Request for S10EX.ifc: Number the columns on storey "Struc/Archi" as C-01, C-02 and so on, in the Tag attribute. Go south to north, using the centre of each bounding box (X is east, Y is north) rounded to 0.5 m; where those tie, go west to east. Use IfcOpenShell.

First a look at what the model holds.

```python
import ifcopenshell
import ifcopenshell.util.element
import ifcopenshell.util.placement

model = ifcopenshell.open("S10EX.ifc")
print(model.schema)
storey = next(s for s in model.by_type("IfcBuildingStorey") if s.Name == "Struc/Archi")
columns = [e for e in ifcopenshell.util.element.get_decomposition(storey) if e.is_a("IfcColumn")]
for e in sorted(columns, key=lambda e: e.id()):
    origin = ifcopenshell.util.placement.get_local_placement(e.ObjectPlacement)[:3, 3]
    print(e.id(), e.Tag, e.Name, origin.round(2) + 0.0, sep=" | ")
```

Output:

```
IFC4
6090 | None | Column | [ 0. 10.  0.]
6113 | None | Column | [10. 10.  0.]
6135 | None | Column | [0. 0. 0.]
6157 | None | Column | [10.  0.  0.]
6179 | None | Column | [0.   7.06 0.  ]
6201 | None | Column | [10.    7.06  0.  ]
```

```python
import ifcopenshell
import ifcopenshell.geom
import ifcopenshell.util.element
import ifcopenshell.util.shape

model = ifcopenshell.open("S10EX.ifc")
settings = ifcopenshell.geom.settings()
settings.set("use-world-coords", True)


def centre(element):
    shape = ifcopenshell.geom.create_shape(settings, element)
    return ifcopenshell.util.shape.get_bbox_centroid(shape.geometry)


storey = next(s for s in model.by_type("IfcBuildingStorey") if s.Name == "Struc/Archi")
columns = [e for e in ifcopenshell.util.element.get_decomposition(storey) if e.is_a("IfcColumn")]

# Insertion points can sit at a corner or the storey origin, so sort by the geometry (in metres).
centres = {e: centre(e) for e in columns}
columns.sort(key=lambda e: (round(centres[e][1] / 0.5), centres[e][0]))

for i, e in enumerate(columns, start=1):
    number = f"C-{i:02d}"
    e.Tag = number
    print(e.id(), number)

model.write("S10EX-out.ifc")
```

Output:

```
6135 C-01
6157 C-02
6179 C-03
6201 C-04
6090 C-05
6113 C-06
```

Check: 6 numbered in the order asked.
